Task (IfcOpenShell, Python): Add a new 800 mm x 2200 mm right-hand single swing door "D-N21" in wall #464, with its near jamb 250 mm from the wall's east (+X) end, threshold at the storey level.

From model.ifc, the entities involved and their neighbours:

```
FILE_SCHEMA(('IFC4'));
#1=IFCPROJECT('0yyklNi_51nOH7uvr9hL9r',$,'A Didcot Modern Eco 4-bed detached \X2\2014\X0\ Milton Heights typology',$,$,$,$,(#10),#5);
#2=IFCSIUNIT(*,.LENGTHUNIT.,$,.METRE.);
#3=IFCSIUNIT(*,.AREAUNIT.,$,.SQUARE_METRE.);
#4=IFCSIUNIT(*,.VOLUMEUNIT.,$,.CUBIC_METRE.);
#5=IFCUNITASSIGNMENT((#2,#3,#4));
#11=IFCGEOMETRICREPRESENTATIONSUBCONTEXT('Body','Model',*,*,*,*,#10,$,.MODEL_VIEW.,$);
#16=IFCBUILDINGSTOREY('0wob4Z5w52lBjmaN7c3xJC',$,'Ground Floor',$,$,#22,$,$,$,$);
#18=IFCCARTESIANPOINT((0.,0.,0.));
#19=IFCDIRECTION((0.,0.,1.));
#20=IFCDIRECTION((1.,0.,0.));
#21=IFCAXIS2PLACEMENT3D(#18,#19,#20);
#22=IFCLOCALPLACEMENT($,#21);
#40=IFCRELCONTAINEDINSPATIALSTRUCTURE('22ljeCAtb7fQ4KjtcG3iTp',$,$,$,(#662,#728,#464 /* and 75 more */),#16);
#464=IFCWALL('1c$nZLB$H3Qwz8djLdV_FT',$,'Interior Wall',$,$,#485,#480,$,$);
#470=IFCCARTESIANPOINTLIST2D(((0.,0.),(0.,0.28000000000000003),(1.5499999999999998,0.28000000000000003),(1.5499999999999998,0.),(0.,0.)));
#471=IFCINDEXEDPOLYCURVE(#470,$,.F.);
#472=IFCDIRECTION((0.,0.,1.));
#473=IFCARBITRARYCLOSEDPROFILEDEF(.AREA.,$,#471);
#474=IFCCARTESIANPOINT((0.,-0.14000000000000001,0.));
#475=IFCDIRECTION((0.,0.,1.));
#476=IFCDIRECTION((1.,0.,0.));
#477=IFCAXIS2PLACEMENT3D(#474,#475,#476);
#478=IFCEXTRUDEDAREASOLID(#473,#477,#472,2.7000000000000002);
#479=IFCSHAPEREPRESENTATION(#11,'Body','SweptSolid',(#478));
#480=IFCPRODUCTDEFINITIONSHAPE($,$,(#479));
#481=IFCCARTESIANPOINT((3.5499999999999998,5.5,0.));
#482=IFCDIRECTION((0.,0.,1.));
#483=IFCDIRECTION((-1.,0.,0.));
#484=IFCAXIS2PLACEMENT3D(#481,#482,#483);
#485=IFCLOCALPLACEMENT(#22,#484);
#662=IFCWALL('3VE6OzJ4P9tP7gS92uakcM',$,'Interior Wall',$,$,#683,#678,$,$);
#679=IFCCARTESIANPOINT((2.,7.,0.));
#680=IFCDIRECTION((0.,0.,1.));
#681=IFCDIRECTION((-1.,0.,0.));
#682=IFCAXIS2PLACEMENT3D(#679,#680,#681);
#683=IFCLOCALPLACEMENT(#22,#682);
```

```python
import numpy as np
import ifcopenshell
import ifcopenshell.api.feature
import ifcopenshell.api.geometry
import ifcopenshell.api.root
import ifcopenshell.api.spatial
import ifcopenshell.geom
import ifcopenshell.util.element
import ifcopenshell.util.placement
import ifcopenshell.util.representation
import ifcopenshell.util.shape
import ifcopenshell.util.unit

model = ifcopenshell.open("model.ifc")
unit_scale = ifcopenshell.util.unit.calculate_unit_scale(model)
settings = ifcopenshell.geom.settings()


def volume(element):
    """Net volume in cubic metres, openings subtracted."""
    shape = ifcopenshell.geom.create_shape(settings, element)
    return ifcopenshell.util.shape.get_volume(shape.geometry)


wall = model.by_id(464)
storey = ifcopenshell.util.element.get_container(wall, ifc_class="IfcBuildingStorey")
context = ifcopenshell.util.representation.get_context(model, "Model", "Body", "MODEL_VIEW")
before = volume(wall)

width, height, from_end, sill = 0.8, 2.2, 0.25, 0.0  # metres

# The wall runs along its own X axis, and the end named is its -X end.
wall_shape = ifcopenshell.geom.create_shape(settings, wall)
x, y, z = ifcopenshell.util.shape.get_vertices(wall_shape.geometry).T
start = x.min() + from_end
face, thickness = float(y.min()), float(y.max() - y.min())
wall_matrix = ifcopenshell.util.placement.get_local_placement(wall.ObjectPlacement)
level = ifcopenshell.util.placement.get_local_placement(storey.ObjectPlacement)[2, 3]


def in_wall(x, y):
    """Placement at x, y metres in the wall's axes, at sill height."""
    matrix = wall_matrix.copy()
    matrix[:, 3] = wall_matrix @ np.array([x / unit_scale, y / unit_scale, 0.0, 1.0])
    matrix[2, 3] = level + sill / unit_scale
    return matrix


# Opening: a box that overshoots both wall faces by 50 mm.
opening = ifcopenshell.api.root.create_entity(model, ifc_class="IfcOpeningElement", predefined_type="OPENING")
box = ifcopenshell.api.geometry.add_wall_representation(
    model, context=context, length=width, height=height, thickness=thickness + 0.1
)
ifcopenshell.api.geometry.assign_representation(model, product=opening, representation=box)
ifcopenshell.api.geometry.edit_object_placement(model, product=opening, matrix=in_wall(start, face - 0.05), is_si=False)
ifcopenshell.api.feature.add_feature(model, feature=opening, element=wall)

door = ifcopenshell.api.root.create_entity(model, ifc_class="IfcDoor", name="D-N21", predefined_type="DOOR")
door.OverallWidth, door.OverallHeight = width / unit_scale, height / unit_scale
door.OperationType = "SINGLE_SWING_RIGHT"
body = ifcopenshell.api.geometry.add_door_representation(
    model,
    context=context,
    overall_width=door.OverallWidth,
    overall_height=door.OverallHeight,
    operation_type="SINGLE_SWING_RIGHT",
    lining_properties={"LiningDepth": thickness / unit_scale, "ThresholdDepth": thickness / unit_scale},
)
ifcopenshell.api.geometry.assign_representation(model, product=door, representation=body)
ifcopenshell.api.spatial.assign_container(model, products=[door], relating_structure=storey)
ifcopenshell.api.feature.add_filling(model, opening=opening, element=door)

# The lining spans the wall, so the door starts at the wall face.
ifcopenshell.api.geometry.edit_object_placement(model, product=door, matrix=in_wall(start, face), is_si=False)

after = volume(wall)

print(f"wall volume {before:.3f} -> {after:.3f} m3")

model.write("model_v2.ifc")
```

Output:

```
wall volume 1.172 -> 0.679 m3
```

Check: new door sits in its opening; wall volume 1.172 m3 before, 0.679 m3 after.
